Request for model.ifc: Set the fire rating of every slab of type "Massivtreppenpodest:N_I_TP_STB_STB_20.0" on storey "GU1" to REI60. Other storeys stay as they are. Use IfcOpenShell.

First a look at what the model holds.

```python
import ifcopenshell
import ifcopenshell.util.element

model = ifcopenshell.open("model.ifc")
print(model.schema)
storey = next(s for s in model.by_type("IfcBuildingStorey") if s.Name == "GU1")
slabs = [e for e in ifcopenshell.util.element.get_decomposition(storey) if e.is_a("IfcSlab")]
seen = {}
for e in slabs:
    element_type = ifcopenshell.util.element.get_type(e)
    key = (element_type.Name if element_type != e and element_type else None, ifcopenshell.util.element.get_pset(e, "Pset_SlabCommon", "FireRating"))
    seen[key] = seen.get(key, 0) + 1
for (name, value), count in sorted(seen.items(), key=str):
    print(count, "x", name, "|", value)
```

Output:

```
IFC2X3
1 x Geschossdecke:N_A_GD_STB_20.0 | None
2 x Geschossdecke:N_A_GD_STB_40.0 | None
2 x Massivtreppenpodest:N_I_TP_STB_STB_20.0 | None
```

```python
import ifcopenshell
import ifcopenshell.api.pset
import ifcopenshell.util.element

model = ifcopenshell.open("model.ifc")

storey = next(s for s in model.by_type("IfcBuildingStorey") if s.Name == "GU1")
slabs = [e for e in ifcopenshell.util.element.get_decomposition(storey) if e.is_a("IfcSlab")]

count = 0
for e in slabs:
    element_type = ifcopenshell.util.element.get_type(e)
    if element_type in (None, e) or element_type.Name != "Massivtreppenpodest:N_I_TP_STB_STB_20.0":
        continue
    found = ifcopenshell.util.element.get_pset(e, "Pset_SlabCommon", should_inherit=False)
    if found:
        pset = model.by_id(found["id"])
        if len(ifcopenshell.util.element.get_elements_by_pset(pset)) > 1:
            pset = ifcopenshell.api.pset.unshare_pset(model, products=[e], pset=pset)[0]
    else:
        pset = ifcopenshell.api.pset.add_pset(model, product=e, name="Pset_SlabCommon")
    ifcopenshell.api.pset.edit_pset(model, pset=pset, properties={"FireRating": "REI60"})
    count += 1

print(count, "slabs updated")

model.write("model_v2.ifc")
```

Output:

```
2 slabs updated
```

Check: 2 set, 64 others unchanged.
